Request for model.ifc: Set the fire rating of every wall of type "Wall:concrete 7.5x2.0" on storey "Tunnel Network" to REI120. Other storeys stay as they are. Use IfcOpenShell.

First a look at what the model holds.

```python
import ifcopenshell
import ifcopenshell.util.element

model = ifcopenshell.open("model.ifc")
print(model.schema)
storey = next(s for s in model.by_type("IfcBuildingStorey") if s.Name == "Tunnel Network")
walls = [e for e in ifcopenshell.util.element.get_decomposition(storey) if e.is_a("IfcWall")]
seen = {}
for e in walls:
    element_type = ifcopenshell.util.element.get_type(e)
    key = (element_type.Name if element_type != e and element_type else None, ifcopenshell.util.element.get_pset(e, "Pset_WallCommon", "FireRating"))
    seen[key] = seen.get(key, 0) + 1
for (name, value), count in sorted(seen.items(), key=str):
    print(count, "x", name, "|", value)
```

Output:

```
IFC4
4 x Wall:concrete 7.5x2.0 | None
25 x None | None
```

```python
import ifcopenshell
import ifcopenshell.api.pset
import ifcopenshell.util.element

model = ifcopenshell.open("model.ifc")

storey = next(s for s in model.by_type("IfcBuildingStorey") if s.Name == "Tunnel Network")
walls = [e for e in ifcopenshell.util.element.get_decomposition(storey) if e.is_a("IfcWall")]

count = 0
for e in walls:
    element_type = ifcopenshell.util.element.get_type(e)
    if element_type in (None, e) or element_type.Name != "Wall:concrete 7.5x2.0":
        continue
    # add_pset returns the element's existing set when there is one.
    pset = ifcopenshell.api.pset.add_pset(model, product=e, name="Pset_WallCommon")
    ifcopenshell.api.pset.edit_pset(model, pset=pset, properties={"FireRating": "REI120"})
    count += 1

print(count, "walls updated")

model.write("model_rev.ifc")
```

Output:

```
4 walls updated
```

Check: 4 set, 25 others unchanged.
